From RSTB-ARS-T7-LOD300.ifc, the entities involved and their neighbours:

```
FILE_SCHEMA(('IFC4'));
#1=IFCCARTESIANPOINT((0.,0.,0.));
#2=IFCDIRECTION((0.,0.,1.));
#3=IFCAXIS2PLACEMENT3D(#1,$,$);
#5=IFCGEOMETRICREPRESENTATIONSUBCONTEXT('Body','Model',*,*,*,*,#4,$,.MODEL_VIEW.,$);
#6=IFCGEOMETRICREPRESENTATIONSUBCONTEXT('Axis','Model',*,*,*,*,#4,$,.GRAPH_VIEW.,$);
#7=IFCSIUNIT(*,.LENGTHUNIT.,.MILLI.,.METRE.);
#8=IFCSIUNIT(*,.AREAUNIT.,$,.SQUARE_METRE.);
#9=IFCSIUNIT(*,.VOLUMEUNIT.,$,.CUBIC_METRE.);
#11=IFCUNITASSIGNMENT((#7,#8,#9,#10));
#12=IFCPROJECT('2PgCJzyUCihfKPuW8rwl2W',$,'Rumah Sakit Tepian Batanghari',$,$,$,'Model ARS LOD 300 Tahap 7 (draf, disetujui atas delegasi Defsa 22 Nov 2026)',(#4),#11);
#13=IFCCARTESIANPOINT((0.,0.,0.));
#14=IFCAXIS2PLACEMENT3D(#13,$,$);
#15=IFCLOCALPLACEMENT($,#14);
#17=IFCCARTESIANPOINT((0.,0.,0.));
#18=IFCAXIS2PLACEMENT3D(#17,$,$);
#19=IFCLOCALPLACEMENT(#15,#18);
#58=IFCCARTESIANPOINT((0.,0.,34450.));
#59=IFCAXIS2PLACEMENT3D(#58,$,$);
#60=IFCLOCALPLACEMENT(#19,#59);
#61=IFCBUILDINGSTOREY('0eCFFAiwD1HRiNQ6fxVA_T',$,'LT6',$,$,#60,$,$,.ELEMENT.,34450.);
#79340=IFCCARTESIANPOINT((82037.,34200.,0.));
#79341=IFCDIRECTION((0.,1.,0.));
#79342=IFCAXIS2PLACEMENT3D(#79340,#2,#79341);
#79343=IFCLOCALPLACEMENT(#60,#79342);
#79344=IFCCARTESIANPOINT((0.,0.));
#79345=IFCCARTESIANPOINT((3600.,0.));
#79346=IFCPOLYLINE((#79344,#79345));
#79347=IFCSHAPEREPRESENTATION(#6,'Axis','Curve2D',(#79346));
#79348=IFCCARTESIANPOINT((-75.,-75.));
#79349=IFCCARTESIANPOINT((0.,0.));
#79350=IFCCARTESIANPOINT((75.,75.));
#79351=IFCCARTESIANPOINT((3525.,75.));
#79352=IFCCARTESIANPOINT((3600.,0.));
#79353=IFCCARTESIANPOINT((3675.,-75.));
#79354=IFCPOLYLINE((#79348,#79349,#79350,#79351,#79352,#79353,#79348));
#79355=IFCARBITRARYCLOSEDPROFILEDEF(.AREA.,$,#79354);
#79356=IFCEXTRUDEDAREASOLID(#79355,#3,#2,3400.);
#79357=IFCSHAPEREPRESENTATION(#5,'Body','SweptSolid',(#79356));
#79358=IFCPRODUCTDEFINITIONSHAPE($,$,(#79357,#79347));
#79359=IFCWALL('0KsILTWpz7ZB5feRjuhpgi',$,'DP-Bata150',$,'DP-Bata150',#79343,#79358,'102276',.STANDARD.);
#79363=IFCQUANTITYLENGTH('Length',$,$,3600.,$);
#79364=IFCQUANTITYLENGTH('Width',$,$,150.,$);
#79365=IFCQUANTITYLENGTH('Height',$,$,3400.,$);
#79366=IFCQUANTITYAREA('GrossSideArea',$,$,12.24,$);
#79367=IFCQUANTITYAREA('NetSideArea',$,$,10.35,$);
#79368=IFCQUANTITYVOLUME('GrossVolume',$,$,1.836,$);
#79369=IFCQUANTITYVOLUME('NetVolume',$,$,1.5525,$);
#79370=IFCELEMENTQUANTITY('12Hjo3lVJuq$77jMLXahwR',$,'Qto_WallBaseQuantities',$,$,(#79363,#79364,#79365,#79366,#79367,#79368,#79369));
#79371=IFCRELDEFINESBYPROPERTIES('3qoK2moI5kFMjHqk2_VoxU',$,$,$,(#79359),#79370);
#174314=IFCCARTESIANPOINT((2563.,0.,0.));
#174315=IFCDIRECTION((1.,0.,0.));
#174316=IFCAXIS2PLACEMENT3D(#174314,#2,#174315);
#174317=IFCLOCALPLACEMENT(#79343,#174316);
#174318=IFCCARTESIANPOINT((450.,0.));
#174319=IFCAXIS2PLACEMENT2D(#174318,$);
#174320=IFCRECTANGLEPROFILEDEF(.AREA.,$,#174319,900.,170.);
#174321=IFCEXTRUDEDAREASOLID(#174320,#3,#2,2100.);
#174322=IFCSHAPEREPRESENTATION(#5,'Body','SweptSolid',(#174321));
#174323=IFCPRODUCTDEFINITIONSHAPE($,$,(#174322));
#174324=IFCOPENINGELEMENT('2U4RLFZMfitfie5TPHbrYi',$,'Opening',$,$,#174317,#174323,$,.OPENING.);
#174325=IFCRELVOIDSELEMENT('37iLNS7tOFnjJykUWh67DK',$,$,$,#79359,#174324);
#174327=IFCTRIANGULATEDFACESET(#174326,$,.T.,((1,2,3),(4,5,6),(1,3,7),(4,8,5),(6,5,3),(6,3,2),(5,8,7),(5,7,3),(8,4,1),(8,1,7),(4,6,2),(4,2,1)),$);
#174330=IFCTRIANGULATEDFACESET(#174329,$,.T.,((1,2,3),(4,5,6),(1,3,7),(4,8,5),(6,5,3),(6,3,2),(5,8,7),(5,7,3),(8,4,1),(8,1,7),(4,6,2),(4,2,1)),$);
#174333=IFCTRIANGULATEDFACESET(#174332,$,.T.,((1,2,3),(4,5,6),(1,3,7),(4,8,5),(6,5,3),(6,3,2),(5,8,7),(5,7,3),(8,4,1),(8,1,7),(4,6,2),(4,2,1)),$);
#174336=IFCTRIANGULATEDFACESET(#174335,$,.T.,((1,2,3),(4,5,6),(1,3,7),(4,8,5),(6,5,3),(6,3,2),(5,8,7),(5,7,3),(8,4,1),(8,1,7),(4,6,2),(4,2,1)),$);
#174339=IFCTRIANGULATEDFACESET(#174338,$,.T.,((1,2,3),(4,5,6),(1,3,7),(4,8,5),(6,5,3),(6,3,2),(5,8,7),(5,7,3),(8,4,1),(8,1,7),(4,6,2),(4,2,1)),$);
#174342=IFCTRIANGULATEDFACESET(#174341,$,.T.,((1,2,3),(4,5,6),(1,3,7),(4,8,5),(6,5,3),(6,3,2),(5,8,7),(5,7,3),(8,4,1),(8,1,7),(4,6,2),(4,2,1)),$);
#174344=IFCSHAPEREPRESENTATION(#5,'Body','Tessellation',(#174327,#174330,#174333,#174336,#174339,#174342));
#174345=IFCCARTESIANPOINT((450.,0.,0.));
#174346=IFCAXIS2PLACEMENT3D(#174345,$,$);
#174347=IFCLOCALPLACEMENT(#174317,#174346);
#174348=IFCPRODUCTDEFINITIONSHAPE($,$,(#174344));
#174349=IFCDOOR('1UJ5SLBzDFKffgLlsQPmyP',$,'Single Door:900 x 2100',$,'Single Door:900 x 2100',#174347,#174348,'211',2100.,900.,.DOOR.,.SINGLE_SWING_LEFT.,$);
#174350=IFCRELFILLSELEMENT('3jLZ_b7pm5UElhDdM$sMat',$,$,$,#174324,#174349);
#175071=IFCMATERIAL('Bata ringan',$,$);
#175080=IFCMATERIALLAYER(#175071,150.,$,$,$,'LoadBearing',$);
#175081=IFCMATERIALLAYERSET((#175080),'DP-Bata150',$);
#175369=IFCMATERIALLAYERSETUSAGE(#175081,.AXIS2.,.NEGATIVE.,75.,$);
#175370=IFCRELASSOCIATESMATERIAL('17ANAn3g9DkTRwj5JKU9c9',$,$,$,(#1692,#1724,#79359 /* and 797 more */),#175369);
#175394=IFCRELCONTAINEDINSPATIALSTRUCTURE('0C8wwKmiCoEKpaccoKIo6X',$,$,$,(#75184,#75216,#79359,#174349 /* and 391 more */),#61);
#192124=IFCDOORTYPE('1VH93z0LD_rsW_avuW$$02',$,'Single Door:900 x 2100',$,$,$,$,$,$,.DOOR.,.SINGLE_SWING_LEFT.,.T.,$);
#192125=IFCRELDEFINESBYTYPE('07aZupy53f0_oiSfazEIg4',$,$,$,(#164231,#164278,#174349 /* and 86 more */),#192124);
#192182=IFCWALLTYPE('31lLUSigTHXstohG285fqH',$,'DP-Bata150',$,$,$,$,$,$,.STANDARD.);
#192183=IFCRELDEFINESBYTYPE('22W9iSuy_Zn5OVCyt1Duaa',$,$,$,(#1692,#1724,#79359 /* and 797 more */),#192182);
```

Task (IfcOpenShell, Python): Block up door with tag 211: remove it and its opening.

```python
import ifcopenshell
import ifcopenshell.api.feature
import ifcopenshell.api.pset
import ifcopenshell.api.root
import ifcopenshell.geom
import ifcopenshell.util.element
import ifcopenshell.util.shape
import ifcopenshell.util.unit

model = ifcopenshell.open("RSTB-ARS-T7-LOD300.ifc")
area_scale = ifcopenshell.util.unit.calculate_unit_scale(model, "AREAUNIT")
volume_scale = ifcopenshell.util.unit.calculate_unit_scale(model, "VOLUMEUNIT")
settings = ifcopenshell.geom.settings()


def volume(element):
    """Net volume in cubic metres, openings subtracted."""
    shape = ifcopenshell.geom.create_shape(settings, element)
    return ifcopenshell.util.shape.get_volume(shape.geometry)


door = model.by_guid("1UJ5SLBzDFKffgLlsQPmyP")
opening = door.FillsVoids[0].RelatingOpeningElement
wall = opening.VoidsElements[0].RelatingBuildingElement
before = volume(wall)

ifcopenshell.api.root.remove_product(model, product=door)
ifcopenshell.api.feature.remove_feature(model, feature=opening)

after = volume(wall)
thickness = 0.15  # wall thickness in metres

# Update the wall's stored quantities.
qto = model.by_id(ifcopenshell.util.element.get_pset(wall, "Qto_WallBaseQuantities", should_inherit=False)["id"])
ifcopenshell.api.pset.edit_qto(model, qto=qto, properties={
    "NetSideArea": after / thickness / area_scale,
    "NetVolume": after / volume_scale,
})

print(f"wall volume {before:.3f} -> {after:.3f} m3")

model.write("RSTB-ARS-T7-LOD300_rev.ifc")
```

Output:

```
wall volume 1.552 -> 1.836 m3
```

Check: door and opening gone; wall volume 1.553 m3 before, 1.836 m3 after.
